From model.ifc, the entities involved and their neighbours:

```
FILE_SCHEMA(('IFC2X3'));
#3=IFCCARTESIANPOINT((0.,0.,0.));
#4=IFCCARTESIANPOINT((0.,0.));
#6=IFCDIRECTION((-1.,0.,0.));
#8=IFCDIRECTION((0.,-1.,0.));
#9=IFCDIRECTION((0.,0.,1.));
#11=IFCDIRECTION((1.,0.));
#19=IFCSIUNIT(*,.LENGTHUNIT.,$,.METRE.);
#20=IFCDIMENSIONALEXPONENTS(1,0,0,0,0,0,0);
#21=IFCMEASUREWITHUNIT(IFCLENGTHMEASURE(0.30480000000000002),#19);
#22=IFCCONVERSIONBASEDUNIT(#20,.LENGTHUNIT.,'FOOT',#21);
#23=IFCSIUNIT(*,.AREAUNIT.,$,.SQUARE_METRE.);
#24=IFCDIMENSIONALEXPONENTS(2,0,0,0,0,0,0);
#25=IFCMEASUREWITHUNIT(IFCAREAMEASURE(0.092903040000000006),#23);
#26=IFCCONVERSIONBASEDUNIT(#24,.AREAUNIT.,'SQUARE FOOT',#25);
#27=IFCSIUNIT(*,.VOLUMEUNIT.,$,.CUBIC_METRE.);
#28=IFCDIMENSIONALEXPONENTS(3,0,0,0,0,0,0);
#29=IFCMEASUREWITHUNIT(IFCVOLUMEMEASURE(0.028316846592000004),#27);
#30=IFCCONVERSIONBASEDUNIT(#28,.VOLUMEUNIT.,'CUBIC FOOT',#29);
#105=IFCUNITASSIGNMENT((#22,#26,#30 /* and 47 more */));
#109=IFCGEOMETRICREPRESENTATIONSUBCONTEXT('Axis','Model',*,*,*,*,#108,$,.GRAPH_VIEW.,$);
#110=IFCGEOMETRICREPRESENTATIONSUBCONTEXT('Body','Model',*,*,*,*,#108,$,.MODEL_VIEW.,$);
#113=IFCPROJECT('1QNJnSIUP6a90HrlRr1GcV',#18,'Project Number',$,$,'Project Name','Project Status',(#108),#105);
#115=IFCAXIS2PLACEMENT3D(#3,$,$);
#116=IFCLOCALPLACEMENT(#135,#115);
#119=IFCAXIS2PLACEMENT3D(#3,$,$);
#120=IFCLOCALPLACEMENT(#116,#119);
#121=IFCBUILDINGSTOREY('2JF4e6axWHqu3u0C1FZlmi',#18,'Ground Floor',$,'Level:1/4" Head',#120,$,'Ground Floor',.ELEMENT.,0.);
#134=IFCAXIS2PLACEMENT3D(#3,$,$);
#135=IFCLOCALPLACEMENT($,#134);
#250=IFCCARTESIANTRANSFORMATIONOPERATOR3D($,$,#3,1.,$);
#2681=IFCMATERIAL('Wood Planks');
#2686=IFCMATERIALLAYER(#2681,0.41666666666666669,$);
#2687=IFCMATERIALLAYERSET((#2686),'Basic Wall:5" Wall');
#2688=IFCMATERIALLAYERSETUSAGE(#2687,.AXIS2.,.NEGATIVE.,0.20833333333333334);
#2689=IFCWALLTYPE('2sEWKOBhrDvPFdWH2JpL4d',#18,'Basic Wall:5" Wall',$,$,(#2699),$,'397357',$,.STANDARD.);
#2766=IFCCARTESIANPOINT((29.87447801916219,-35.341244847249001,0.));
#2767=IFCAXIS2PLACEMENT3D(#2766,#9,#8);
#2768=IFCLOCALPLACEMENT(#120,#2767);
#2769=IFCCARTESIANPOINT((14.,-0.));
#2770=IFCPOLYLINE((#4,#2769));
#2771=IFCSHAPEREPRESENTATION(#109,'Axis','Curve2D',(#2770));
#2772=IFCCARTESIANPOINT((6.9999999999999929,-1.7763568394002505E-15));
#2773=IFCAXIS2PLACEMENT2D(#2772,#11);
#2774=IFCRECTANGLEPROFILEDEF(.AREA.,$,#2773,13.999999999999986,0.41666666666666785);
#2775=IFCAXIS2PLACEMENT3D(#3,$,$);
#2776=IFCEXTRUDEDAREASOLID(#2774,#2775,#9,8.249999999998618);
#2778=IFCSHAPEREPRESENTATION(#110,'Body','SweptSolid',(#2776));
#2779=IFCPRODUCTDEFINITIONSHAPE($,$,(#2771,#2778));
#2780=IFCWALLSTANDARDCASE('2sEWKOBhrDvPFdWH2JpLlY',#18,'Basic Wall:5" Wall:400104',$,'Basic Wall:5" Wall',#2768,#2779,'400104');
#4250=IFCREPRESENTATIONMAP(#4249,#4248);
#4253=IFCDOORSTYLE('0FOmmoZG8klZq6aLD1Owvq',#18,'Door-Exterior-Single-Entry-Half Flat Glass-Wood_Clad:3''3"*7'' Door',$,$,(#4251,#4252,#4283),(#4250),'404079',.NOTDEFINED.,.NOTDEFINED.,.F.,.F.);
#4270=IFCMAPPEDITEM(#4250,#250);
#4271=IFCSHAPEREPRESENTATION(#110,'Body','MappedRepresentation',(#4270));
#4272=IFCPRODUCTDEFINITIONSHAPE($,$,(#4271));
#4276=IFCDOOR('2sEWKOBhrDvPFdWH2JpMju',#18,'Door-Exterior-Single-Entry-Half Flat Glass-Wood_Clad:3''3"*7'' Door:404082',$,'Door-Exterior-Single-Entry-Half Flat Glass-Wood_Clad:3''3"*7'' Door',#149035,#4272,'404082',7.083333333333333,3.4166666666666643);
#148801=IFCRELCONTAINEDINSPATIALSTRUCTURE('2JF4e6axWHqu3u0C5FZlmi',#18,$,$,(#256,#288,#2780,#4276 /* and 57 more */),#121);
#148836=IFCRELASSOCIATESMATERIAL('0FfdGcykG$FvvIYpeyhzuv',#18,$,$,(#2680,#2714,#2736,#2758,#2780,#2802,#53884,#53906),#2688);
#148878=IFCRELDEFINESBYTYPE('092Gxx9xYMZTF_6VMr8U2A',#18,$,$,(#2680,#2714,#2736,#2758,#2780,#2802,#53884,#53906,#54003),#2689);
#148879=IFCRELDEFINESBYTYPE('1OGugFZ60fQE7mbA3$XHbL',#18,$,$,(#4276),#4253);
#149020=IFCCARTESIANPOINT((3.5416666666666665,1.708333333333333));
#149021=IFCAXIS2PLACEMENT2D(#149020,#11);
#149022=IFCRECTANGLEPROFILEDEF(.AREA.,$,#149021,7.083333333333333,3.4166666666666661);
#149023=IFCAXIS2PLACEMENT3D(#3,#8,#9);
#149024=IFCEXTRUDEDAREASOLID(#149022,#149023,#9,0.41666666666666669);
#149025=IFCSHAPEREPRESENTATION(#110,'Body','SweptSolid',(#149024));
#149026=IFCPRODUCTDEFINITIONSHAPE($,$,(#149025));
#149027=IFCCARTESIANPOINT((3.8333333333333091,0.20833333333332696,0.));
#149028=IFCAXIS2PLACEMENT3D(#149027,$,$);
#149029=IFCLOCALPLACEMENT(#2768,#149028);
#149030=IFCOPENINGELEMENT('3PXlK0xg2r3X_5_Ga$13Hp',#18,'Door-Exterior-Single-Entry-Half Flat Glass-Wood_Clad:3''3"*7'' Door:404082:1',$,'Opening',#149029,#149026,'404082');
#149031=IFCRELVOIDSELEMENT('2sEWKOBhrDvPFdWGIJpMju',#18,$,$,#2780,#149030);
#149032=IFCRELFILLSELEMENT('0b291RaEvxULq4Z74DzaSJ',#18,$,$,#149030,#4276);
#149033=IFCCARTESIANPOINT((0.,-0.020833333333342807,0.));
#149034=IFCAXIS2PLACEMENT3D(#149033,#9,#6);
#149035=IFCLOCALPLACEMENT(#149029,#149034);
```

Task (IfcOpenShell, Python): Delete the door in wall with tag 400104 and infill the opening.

```python
import ifcopenshell
import ifcopenshell.api.feature
import ifcopenshell.api.root
import ifcopenshell.geom
import ifcopenshell.util.shape

model = ifcopenshell.open("model.ifc")
settings = ifcopenshell.geom.settings()


def volume(element):
    """Net volume in cubic metres, openings subtracted."""
    shape = ifcopenshell.geom.create_shape(settings, element)
    return ifcopenshell.util.shape.get_volume(shape.geometry)


door = model.by_guid("2sEWKOBhrDvPFdWH2JpMju")
opening = door.FillsVoids[0].RelatingOpeningElement
wall = opening.VoidsElements[0].RelatingBuildingElement
before = volume(wall)

ifcopenshell.api.root.remove_product(model, product=door)
ifcopenshell.api.feature.remove_feature(model, feature=opening)

after = volume(wall)

print(f"wall volume {before:.3f} -> {after:.3f} m3")

model.write("model_v2.ifc")
```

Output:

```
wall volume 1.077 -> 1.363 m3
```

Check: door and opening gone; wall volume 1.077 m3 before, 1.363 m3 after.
